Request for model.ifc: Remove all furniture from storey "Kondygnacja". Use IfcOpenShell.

First a look at what the model holds.

```python
import ifcopenshell
import ifcopenshell.util.element

model = ifcopenshell.open("model.ifc")
print(model.schema)
storey = next(s for s in model.by_type("IfcBuildingStorey") if s.Name == "Kondygnacja")
furniture = [e for e in ifcopenshell.util.element.get_decomposition(storey) if e.is_a("IfcFurnishingElement")]
seen = {}
for e in furniture:
    element_type = ifcopenshell.util.element.get_type(e)
    name = element_type.Name if element_type not in (None, e) else None
    seen[name] = seen.get(name, 0) + 1
for name, count in sorted(seen.items(), key=str):
    print(count, "x", name)
```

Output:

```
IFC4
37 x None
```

```python
import ifcopenshell
import ifcopenshell.api.root
import ifcopenshell.util.element

model = ifcopenshell.open("model.ifc")

storey = next(s for s in model.by_type("IfcBuildingStorey") if s.Name == "Kondygnacja")
furniture = [e for e in ifcopenshell.util.element.get_decomposition(storey) if e.is_a("IfcFurnishingElement")]

for e in furniture:
    ifcopenshell.api.root.remove_product(model, product=e)
print(len(furniture), "removed")

model.write("model_updated.ifc")
```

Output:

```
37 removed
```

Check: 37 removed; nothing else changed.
